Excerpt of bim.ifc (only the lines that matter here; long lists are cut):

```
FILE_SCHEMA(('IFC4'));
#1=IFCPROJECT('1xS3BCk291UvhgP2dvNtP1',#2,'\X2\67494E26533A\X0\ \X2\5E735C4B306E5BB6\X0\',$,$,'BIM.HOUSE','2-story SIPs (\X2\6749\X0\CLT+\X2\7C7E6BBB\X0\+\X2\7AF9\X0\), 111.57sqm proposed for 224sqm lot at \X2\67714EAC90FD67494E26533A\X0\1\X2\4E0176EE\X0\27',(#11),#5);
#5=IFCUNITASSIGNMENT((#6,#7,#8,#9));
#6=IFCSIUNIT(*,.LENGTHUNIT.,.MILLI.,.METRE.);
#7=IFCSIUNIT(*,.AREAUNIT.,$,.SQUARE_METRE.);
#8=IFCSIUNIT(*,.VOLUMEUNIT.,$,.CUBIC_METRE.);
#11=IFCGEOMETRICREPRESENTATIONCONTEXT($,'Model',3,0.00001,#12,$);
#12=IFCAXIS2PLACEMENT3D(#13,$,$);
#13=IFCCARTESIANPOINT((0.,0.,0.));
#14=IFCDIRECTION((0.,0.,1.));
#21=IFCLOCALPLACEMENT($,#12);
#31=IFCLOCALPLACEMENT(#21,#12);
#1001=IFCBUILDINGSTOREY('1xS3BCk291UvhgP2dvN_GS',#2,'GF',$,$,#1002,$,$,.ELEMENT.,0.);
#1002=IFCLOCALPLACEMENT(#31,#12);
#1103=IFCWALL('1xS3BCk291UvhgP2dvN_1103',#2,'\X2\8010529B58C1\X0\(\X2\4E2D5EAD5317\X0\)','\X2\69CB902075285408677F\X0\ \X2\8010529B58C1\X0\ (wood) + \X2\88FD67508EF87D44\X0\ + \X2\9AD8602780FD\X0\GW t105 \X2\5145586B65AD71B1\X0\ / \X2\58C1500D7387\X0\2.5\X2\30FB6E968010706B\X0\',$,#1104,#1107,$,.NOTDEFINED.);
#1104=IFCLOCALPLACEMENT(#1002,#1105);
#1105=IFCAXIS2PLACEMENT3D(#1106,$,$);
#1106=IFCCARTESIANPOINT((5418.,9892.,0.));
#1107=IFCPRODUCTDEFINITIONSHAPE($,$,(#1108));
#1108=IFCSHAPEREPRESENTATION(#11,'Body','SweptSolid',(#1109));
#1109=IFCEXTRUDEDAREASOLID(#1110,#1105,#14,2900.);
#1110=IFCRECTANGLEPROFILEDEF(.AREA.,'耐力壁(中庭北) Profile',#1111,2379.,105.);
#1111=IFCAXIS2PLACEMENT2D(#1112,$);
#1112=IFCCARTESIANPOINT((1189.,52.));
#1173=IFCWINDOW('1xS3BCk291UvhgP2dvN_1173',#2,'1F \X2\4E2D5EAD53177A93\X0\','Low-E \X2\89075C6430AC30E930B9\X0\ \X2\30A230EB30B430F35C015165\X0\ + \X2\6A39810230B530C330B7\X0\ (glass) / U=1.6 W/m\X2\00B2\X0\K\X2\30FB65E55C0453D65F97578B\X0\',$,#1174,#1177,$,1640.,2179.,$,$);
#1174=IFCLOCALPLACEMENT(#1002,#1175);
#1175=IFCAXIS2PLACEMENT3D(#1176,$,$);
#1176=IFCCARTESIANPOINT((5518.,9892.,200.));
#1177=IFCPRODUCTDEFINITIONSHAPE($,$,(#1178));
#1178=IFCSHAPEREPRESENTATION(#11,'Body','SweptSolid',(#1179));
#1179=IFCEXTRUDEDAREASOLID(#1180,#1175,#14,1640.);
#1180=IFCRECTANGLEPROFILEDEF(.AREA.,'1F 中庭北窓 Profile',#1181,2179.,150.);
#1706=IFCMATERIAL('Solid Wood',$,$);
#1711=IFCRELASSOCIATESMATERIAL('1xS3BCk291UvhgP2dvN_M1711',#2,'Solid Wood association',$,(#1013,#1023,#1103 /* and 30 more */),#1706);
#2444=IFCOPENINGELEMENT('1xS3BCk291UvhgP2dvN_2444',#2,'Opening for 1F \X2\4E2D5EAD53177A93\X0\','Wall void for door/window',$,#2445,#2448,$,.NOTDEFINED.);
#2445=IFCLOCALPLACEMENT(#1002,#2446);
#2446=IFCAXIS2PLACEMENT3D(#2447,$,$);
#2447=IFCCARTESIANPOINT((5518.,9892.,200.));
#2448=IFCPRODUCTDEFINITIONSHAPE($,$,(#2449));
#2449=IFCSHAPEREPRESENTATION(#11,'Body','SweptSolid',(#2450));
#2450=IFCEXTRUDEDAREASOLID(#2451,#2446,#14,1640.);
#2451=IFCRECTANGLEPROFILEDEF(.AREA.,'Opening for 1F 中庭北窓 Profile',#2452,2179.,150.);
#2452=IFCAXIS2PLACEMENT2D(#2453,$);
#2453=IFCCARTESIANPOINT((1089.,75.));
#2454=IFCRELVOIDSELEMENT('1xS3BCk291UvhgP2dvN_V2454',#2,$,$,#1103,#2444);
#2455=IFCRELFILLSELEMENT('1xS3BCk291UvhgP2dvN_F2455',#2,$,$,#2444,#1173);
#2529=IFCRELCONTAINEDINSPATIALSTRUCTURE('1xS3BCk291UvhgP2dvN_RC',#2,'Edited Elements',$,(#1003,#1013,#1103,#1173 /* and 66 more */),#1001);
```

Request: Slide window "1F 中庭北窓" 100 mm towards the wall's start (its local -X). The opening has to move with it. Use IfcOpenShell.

```python
import ifcopenshell
import ifcopenshell.api.geometry
import ifcopenshell.util.placement

model = ifcopenshell.open("bim.ifc")

window = model.by_id(1173)
opening = window.FillsVoids[0].RelatingOpeningElement
wall = opening.VoidsElements[0].RelatingBuildingElement

wall_matrix = ifcopenshell.util.placement.get_local_placement(wall.ObjectPlacement)
shift = wall_matrix[:3, 0] * -100.0
before = ifcopenshell.util.placement.get_local_placement(window.ObjectPlacement)[:3, 3].copy()

# The window is not placed relative to its opening, so move both.
for product in (opening, window):
    matrix = ifcopenshell.util.placement.get_local_placement(product.ObjectPlacement)
    matrix[:3, 3] += shift
    ifcopenshell.api.geometry.edit_object_placement(model, product=product, matrix=matrix, is_si=False)

after = ifcopenshell.util.placement.get_local_placement(window.ObjectPlacement)[:3, 3]
print("window moved by", (after - before).round(3) + 0.0)

model.write("bim_edited.ifc")
```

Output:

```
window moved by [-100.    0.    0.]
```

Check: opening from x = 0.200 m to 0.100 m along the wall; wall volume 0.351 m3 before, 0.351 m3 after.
